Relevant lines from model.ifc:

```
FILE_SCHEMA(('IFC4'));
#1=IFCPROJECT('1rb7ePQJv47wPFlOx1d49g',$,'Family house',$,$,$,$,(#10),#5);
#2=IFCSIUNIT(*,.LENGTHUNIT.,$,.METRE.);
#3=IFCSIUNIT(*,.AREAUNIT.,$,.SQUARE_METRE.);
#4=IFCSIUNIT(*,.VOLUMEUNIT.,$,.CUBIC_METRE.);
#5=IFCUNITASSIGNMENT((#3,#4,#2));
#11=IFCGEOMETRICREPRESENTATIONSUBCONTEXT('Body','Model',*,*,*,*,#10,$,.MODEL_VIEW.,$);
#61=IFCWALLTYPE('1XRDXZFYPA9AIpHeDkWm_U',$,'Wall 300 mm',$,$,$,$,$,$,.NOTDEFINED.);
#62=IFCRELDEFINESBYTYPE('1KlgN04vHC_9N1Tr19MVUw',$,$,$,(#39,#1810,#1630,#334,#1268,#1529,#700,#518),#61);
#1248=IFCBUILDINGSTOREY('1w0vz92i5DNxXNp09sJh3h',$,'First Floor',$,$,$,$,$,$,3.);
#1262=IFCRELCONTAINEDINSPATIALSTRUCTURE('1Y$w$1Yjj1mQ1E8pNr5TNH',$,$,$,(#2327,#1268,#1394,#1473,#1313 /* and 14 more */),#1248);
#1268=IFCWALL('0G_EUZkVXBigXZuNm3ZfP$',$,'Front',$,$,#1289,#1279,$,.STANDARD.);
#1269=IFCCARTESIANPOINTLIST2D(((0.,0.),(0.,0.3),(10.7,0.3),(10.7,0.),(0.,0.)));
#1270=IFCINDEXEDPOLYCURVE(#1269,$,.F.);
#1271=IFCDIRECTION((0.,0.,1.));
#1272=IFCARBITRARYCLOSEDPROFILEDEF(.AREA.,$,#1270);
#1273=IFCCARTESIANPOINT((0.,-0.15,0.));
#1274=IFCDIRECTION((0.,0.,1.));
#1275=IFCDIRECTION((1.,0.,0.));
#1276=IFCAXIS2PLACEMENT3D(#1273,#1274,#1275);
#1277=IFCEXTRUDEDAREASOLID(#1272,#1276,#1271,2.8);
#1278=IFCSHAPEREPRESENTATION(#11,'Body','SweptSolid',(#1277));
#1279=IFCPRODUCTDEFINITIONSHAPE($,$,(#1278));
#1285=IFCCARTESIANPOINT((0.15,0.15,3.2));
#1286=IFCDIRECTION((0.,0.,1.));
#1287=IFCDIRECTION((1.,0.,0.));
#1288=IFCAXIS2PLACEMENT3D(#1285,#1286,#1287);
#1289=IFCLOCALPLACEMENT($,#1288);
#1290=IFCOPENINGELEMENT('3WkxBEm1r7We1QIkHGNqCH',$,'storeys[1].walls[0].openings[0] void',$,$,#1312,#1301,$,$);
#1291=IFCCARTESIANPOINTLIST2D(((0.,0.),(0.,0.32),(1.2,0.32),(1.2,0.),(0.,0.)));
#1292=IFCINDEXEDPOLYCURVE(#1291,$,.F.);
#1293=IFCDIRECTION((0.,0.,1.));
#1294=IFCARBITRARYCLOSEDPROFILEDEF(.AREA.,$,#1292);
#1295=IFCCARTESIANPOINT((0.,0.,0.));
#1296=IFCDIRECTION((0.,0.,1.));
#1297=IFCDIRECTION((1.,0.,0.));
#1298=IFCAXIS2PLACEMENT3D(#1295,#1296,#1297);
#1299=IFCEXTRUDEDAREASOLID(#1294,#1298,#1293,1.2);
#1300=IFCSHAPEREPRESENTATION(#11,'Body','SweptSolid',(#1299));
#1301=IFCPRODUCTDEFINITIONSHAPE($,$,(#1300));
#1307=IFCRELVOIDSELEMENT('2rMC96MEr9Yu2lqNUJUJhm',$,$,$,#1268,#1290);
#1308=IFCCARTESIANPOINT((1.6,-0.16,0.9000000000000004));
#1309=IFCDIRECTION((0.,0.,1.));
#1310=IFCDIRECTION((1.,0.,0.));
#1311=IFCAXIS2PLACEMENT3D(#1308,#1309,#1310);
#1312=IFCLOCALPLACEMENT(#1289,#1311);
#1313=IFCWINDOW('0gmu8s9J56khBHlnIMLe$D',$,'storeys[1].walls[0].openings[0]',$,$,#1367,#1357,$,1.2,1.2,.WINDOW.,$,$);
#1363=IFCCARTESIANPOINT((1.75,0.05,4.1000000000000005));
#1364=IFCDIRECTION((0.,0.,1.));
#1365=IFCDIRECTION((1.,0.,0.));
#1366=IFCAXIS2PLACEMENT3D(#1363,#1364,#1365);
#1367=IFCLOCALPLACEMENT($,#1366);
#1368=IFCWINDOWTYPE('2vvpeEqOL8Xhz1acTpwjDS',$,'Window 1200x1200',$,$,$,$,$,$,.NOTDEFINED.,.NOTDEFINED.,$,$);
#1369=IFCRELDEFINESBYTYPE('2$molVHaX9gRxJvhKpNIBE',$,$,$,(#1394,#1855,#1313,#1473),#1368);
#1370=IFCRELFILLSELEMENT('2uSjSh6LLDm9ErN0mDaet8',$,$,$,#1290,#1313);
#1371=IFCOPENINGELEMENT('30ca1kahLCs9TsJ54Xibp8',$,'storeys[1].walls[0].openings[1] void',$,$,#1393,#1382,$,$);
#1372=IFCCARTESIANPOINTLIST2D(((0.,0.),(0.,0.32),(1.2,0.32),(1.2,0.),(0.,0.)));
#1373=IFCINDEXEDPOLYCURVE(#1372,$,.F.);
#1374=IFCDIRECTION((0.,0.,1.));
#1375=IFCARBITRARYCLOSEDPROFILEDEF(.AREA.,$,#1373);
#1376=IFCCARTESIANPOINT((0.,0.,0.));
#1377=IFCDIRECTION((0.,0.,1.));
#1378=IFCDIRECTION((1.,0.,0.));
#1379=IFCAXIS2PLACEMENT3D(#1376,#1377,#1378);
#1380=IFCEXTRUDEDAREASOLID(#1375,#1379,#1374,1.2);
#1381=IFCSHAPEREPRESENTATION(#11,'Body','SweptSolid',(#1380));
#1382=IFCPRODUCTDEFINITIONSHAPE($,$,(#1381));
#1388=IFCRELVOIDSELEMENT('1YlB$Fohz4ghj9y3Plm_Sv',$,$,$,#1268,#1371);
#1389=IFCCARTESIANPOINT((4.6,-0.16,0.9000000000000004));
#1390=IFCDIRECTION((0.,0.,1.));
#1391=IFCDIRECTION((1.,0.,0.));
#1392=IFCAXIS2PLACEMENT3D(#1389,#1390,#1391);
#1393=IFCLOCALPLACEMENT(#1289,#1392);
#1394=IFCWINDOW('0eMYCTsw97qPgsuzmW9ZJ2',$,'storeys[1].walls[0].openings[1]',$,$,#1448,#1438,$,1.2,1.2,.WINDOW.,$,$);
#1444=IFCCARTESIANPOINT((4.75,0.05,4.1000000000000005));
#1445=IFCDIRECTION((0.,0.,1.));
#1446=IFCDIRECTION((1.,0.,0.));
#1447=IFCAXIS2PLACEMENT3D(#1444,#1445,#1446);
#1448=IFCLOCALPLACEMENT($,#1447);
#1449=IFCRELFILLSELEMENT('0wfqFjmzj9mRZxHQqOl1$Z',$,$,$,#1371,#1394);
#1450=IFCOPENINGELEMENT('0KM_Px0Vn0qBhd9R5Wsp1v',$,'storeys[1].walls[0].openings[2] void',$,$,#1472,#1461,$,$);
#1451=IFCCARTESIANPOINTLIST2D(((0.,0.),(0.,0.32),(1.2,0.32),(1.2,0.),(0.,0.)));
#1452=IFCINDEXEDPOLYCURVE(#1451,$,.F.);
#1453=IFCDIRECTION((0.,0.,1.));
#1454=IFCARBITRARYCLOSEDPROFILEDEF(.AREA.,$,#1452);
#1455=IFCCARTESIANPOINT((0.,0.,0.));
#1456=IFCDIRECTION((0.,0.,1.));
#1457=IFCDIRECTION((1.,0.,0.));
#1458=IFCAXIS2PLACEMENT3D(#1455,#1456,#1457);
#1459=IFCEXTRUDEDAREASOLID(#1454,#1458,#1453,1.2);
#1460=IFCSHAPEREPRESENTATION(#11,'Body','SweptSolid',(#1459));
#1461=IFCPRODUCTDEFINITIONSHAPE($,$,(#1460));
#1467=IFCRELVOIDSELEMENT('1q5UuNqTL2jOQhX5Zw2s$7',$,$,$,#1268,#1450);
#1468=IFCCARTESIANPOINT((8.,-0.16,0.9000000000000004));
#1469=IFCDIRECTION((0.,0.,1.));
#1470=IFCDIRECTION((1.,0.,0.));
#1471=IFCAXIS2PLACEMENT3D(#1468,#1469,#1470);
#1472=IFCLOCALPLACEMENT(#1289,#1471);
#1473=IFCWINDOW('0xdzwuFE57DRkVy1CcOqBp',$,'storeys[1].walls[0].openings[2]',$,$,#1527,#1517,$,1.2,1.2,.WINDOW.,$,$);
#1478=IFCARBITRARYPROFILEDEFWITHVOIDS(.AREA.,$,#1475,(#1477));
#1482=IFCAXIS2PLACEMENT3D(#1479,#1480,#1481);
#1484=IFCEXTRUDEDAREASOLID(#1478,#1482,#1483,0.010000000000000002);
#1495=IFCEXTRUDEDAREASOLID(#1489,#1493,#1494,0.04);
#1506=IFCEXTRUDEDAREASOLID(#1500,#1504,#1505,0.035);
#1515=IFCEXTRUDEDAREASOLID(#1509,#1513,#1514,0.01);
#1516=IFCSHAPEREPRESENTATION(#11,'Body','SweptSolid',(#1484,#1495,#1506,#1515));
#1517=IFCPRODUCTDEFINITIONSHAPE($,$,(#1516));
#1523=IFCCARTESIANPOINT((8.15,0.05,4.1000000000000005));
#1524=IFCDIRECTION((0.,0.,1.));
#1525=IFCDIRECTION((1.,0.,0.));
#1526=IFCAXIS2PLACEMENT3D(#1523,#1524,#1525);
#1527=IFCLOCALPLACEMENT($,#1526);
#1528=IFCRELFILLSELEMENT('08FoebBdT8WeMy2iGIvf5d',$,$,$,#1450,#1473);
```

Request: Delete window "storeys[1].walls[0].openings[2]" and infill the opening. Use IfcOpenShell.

```python
import ifcopenshell
import ifcopenshell.api.feature
import ifcopenshell.api.root
import ifcopenshell.geom
import ifcopenshell.util.shape

model = ifcopenshell.open("model.ifc")
settings = ifcopenshell.geom.settings()


def volume(element):
    """Net volume in cubic metres, openings subtracted."""
    shape = ifcopenshell.geom.create_shape(settings, element)
    return ifcopenshell.util.shape.get_volume(shape.geometry)


window = model.by_guid("0xdzwuFE57DRkVy1CcOqBp")
opening = window.FillsVoids[0].RelatingOpeningElement
wall = opening.VoidsElements[0].RelatingBuildingElement
before = volume(wall)

ifcopenshell.api.root.remove_product(model, product=window)
ifcopenshell.api.feature.remove_feature(model, feature=opening)

after = volume(wall)

print(f"wall volume {before:.3f} -> {after:.3f} m3")

model.write("model_rev.ifc")
```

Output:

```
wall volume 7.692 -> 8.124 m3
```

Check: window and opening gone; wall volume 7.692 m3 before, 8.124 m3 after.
